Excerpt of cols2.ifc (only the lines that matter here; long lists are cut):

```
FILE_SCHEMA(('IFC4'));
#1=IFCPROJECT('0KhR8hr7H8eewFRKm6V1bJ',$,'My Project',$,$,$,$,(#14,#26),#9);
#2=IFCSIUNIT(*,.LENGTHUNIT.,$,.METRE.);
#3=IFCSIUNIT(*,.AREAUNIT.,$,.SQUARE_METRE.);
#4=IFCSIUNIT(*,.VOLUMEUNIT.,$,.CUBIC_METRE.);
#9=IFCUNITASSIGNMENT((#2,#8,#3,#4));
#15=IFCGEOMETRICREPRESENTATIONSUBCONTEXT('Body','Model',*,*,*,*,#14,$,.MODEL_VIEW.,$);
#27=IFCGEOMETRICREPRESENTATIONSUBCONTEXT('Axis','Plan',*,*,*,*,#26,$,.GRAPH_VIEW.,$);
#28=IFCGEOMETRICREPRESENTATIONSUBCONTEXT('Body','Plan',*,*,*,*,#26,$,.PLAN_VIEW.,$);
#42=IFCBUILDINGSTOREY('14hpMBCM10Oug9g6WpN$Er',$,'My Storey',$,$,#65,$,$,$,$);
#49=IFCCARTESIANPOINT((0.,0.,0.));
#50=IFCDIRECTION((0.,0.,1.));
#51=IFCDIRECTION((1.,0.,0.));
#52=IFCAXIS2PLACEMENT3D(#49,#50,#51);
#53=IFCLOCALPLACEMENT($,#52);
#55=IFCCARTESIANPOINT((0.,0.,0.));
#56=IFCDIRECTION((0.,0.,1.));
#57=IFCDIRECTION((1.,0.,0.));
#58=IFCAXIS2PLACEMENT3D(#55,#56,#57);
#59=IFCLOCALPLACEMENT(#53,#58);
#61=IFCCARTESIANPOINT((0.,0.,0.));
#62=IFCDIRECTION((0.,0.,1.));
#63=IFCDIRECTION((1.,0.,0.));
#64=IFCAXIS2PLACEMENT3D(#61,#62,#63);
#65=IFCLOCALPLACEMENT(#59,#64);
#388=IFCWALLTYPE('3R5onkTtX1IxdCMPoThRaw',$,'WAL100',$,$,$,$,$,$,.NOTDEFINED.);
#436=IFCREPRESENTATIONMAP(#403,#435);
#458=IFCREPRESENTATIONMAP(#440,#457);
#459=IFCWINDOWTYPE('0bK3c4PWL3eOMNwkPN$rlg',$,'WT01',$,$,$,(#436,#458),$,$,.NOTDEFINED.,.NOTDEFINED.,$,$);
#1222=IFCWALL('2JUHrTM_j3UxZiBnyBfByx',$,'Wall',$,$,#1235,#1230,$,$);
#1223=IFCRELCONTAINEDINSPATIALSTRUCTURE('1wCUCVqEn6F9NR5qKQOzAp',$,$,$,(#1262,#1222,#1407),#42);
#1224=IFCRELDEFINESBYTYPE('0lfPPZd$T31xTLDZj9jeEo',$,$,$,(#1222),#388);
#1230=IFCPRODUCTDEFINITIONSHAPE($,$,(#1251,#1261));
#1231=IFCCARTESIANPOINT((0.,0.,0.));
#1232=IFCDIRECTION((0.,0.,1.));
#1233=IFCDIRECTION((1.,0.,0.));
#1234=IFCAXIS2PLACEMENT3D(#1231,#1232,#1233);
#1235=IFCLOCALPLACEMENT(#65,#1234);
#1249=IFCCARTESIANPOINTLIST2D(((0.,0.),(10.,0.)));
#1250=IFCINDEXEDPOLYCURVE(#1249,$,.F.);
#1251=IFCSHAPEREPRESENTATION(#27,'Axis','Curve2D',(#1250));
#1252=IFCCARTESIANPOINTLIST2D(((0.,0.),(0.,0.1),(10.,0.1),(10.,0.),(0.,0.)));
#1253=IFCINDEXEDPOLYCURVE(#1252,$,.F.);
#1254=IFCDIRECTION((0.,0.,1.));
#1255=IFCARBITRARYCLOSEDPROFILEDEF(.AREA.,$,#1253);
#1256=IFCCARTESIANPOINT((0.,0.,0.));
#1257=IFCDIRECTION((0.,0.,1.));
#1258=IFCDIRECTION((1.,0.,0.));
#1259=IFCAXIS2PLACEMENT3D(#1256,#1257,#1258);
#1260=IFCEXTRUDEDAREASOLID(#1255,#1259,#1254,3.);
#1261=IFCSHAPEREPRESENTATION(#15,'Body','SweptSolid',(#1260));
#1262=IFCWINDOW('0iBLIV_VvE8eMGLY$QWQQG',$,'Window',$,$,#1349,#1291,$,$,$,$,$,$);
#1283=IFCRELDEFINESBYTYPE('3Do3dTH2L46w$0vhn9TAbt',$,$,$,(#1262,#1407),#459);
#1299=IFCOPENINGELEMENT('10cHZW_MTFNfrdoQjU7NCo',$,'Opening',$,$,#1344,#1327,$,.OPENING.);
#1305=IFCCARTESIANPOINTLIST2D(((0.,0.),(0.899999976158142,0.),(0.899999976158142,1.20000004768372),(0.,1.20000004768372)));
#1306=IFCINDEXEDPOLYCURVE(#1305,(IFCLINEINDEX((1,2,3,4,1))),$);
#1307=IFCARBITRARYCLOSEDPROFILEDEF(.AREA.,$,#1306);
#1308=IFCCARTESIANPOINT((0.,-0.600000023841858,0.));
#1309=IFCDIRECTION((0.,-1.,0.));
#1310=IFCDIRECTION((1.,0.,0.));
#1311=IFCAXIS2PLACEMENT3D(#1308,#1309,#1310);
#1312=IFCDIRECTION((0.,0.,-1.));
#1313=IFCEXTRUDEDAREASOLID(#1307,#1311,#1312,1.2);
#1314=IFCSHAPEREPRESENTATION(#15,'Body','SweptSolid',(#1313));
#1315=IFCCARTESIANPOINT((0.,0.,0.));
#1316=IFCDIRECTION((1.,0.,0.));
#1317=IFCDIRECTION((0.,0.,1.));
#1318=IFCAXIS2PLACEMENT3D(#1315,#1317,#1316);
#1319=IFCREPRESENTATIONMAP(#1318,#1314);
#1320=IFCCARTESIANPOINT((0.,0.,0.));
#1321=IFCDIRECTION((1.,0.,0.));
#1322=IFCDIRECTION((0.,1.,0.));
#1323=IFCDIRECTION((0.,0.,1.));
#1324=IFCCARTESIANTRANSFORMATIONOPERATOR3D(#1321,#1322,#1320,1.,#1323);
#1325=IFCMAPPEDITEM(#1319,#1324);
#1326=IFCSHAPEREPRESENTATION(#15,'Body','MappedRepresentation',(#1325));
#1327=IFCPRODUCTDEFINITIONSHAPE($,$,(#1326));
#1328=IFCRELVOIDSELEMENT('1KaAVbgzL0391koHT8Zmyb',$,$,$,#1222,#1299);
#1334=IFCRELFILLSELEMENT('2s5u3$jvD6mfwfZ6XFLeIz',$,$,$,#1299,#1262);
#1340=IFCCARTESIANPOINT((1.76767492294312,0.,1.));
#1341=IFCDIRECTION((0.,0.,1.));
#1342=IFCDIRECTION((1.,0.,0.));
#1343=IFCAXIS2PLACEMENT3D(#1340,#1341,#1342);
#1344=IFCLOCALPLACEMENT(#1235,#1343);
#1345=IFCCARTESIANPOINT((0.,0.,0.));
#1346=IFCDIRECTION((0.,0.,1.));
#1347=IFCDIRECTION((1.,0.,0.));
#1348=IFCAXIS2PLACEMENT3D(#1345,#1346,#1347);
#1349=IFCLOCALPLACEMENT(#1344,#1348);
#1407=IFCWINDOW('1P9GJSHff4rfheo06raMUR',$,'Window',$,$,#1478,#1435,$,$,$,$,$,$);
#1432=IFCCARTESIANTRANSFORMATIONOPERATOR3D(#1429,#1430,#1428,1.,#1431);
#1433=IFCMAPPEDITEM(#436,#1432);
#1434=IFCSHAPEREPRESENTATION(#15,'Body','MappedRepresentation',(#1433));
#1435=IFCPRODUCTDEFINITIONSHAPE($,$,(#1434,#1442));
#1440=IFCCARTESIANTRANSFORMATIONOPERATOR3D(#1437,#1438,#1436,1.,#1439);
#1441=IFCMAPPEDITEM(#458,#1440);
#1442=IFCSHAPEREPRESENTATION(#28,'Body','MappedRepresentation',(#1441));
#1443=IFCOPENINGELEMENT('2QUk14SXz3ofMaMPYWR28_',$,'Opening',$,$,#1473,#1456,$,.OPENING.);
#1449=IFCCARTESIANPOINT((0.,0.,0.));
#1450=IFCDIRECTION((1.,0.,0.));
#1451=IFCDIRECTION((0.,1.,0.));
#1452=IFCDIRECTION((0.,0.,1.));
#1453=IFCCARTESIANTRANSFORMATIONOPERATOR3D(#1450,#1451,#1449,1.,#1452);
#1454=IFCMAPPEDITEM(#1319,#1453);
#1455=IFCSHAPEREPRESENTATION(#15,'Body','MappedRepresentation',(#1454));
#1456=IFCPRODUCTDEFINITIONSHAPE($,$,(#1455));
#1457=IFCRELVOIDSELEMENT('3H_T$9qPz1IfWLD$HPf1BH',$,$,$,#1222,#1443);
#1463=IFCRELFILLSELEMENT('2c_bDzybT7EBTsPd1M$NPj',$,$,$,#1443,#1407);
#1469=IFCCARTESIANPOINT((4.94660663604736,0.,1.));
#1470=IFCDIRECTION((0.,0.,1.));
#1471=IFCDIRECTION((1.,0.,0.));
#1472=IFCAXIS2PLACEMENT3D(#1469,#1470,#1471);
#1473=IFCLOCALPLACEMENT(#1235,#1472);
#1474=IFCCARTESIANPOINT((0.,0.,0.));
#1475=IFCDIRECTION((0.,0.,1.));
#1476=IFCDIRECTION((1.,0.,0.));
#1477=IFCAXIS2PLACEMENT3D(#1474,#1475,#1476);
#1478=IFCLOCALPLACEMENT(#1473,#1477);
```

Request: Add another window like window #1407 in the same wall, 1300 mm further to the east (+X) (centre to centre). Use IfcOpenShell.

```python
import ifcopenshell
import ifcopenshell.api.feature
import ifcopenshell.api.geometry
import ifcopenshell.api.root
import ifcopenshell.geom
import ifcopenshell.util.element
import ifcopenshell.util.placement
import ifcopenshell.util.shape
import ifcopenshell.util.unit

model = ifcopenshell.open("cols2.ifc")
unit_scale = ifcopenshell.util.unit.calculate_unit_scale(model)
settings = ifcopenshell.geom.settings()


def volume(element):
    """Net volume in cubic metres, openings subtracted."""
    shape = ifcopenshell.geom.create_shape(settings, element)
    return ifcopenshell.util.shape.get_volume(shape.geometry)


window = model.by_guid("1P9GJSHff4rfheo06raMUR")
opening = window.FillsVoids[0].RelatingOpeningElement
wall = opening.VoidsElements[0].RelatingBuildingElement
before = volume(wall)
shift = ifcopenshell.util.placement.get_local_placement(wall.ObjectPlacement)[:3, 0] * 1.3 / unit_scale

# copy_class copies the void relationship, type, container and properties, but no geometry.
new_opening = ifcopenshell.api.root.copy_class(model, product=opening)
new_opening.Representation = ifcopenshell.util.element.copy_deep(
    model, opening.Representation, exclude=["IfcGeometricRepresentationContext", "IfcRepresentationMap"]
)
new_window = ifcopenshell.api.root.copy_class(model, product=window)
new_window.Representation = ifcopenshell.util.element.copy_deep(
    model, window.Representation, exclude=["IfcGeometricRepresentationContext", "IfcRepresentationMap"]
)
ifcopenshell.api.feature.add_filling(model, opening=new_opening, element=new_window)

for old, new in ((opening, new_opening), (window, new_window)):
    matrix = ifcopenshell.util.placement.get_local_placement(old.ObjectPlacement)
    matrix[:3, 3] += shift
    ifcopenshell.api.geometry.edit_object_placement(model, product=new, matrix=matrix, is_si=False)

after = volume(wall)

print(f"wall volume {before:.3f} -> {after:.3f} m3")

model.write("cols2-out.ifc")
```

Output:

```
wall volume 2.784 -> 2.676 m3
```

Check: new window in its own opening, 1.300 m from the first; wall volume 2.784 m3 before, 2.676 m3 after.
